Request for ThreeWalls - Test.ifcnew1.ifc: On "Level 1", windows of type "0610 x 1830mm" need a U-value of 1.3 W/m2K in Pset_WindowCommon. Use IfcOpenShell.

First a look at what the model holds.

```python
import ifcopenshell
import ifcopenshell.util.element

model = ifcopenshell.open("ThreeWalls - Test.ifcnew1.ifc")
print(model.schema)
storey = next(s for s in model.by_type("IfcBuildingStorey") if s.Name == "Level 1")
windows = [e for e in ifcopenshell.util.element.get_decomposition(storey) if e.is_a("IfcWindow")]
seen = {}
for e in windows:
    element_type = ifcopenshell.util.element.get_type(e)
    key = (element_type.Name if element_type != e and element_type else None, ifcopenshell.util.element.get_pset(e, "Pset_WindowCommon", "ThermalTransmittance"))
    seen[key] = seen.get(key, 0) + 1
for (name, value), count in sorted(seen.items(), key=str):
    print(count, "x", name, "|", value)
```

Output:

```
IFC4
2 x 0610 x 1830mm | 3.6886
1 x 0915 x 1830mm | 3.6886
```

```python
import ifcopenshell
import ifcopenshell.api.pset
import ifcopenshell.util.element

model = ifcopenshell.open("ThreeWalls - Test.ifcnew1.ifc")

storey = next(s for s in model.by_type("IfcBuildingStorey") if s.Name == "Level 1")
windows = [e for e in ifcopenshell.util.element.get_decomposition(storey) if e.is_a("IfcWindow")]

count = 0
for e in windows:
    element_type = ifcopenshell.util.element.get_type(e)
    if element_type in (None, e) or element_type.Name != "0610 x 1830mm":
        continue
    # add_pset returns the element's existing set when there is one.
    pset = ifcopenshell.api.pset.add_pset(model, product=e, name="Pset_WindowCommon")
    ifcopenshell.api.pset.edit_pset(model, pset=pset, properties={"ThermalTransmittance": 1.3})
    count += 1

print(count, "windows updated")

model.write("ThreeWalls - Test.ifcnew1_edited.ifc")
```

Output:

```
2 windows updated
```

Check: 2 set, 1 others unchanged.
